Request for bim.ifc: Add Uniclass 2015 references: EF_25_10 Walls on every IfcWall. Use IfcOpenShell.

First a look at what the model holds.

```python
import ifcopenshell

model = ifcopenshell.open("bim.ifc")
print(model.schema)
print("classifications:", [c.Name for c in model.by_type("IfcClassification")])
for ifc_class in ("IfcDoor", "IfcRoof", "IfcStair", "IfcWall", "IfcWindow"):
    print(ifc_class, len(model.by_type(ifc_class)))
```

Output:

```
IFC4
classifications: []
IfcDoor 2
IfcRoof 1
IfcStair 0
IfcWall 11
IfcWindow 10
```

```python
import ifcopenshell
import ifcopenshell.api.classification

model = ifcopenshell.open("bim.ifc")

system = ifcopenshell.api.classification.add_classification(model, classification="Uniclass 2015")

codes = {
    "IfcWall": ("EF_25_10", "Walls"),
}
for ifc_class, (code, name) in codes.items():
    products = model.by_type(ifc_class)
    ifcopenshell.api.classification.add_reference(
        model, products=products, classification=system, identification=code, name=name
    )
    print(code, len(products))

model.write("bim_v2.ifc")
```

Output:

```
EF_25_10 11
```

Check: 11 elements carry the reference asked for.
